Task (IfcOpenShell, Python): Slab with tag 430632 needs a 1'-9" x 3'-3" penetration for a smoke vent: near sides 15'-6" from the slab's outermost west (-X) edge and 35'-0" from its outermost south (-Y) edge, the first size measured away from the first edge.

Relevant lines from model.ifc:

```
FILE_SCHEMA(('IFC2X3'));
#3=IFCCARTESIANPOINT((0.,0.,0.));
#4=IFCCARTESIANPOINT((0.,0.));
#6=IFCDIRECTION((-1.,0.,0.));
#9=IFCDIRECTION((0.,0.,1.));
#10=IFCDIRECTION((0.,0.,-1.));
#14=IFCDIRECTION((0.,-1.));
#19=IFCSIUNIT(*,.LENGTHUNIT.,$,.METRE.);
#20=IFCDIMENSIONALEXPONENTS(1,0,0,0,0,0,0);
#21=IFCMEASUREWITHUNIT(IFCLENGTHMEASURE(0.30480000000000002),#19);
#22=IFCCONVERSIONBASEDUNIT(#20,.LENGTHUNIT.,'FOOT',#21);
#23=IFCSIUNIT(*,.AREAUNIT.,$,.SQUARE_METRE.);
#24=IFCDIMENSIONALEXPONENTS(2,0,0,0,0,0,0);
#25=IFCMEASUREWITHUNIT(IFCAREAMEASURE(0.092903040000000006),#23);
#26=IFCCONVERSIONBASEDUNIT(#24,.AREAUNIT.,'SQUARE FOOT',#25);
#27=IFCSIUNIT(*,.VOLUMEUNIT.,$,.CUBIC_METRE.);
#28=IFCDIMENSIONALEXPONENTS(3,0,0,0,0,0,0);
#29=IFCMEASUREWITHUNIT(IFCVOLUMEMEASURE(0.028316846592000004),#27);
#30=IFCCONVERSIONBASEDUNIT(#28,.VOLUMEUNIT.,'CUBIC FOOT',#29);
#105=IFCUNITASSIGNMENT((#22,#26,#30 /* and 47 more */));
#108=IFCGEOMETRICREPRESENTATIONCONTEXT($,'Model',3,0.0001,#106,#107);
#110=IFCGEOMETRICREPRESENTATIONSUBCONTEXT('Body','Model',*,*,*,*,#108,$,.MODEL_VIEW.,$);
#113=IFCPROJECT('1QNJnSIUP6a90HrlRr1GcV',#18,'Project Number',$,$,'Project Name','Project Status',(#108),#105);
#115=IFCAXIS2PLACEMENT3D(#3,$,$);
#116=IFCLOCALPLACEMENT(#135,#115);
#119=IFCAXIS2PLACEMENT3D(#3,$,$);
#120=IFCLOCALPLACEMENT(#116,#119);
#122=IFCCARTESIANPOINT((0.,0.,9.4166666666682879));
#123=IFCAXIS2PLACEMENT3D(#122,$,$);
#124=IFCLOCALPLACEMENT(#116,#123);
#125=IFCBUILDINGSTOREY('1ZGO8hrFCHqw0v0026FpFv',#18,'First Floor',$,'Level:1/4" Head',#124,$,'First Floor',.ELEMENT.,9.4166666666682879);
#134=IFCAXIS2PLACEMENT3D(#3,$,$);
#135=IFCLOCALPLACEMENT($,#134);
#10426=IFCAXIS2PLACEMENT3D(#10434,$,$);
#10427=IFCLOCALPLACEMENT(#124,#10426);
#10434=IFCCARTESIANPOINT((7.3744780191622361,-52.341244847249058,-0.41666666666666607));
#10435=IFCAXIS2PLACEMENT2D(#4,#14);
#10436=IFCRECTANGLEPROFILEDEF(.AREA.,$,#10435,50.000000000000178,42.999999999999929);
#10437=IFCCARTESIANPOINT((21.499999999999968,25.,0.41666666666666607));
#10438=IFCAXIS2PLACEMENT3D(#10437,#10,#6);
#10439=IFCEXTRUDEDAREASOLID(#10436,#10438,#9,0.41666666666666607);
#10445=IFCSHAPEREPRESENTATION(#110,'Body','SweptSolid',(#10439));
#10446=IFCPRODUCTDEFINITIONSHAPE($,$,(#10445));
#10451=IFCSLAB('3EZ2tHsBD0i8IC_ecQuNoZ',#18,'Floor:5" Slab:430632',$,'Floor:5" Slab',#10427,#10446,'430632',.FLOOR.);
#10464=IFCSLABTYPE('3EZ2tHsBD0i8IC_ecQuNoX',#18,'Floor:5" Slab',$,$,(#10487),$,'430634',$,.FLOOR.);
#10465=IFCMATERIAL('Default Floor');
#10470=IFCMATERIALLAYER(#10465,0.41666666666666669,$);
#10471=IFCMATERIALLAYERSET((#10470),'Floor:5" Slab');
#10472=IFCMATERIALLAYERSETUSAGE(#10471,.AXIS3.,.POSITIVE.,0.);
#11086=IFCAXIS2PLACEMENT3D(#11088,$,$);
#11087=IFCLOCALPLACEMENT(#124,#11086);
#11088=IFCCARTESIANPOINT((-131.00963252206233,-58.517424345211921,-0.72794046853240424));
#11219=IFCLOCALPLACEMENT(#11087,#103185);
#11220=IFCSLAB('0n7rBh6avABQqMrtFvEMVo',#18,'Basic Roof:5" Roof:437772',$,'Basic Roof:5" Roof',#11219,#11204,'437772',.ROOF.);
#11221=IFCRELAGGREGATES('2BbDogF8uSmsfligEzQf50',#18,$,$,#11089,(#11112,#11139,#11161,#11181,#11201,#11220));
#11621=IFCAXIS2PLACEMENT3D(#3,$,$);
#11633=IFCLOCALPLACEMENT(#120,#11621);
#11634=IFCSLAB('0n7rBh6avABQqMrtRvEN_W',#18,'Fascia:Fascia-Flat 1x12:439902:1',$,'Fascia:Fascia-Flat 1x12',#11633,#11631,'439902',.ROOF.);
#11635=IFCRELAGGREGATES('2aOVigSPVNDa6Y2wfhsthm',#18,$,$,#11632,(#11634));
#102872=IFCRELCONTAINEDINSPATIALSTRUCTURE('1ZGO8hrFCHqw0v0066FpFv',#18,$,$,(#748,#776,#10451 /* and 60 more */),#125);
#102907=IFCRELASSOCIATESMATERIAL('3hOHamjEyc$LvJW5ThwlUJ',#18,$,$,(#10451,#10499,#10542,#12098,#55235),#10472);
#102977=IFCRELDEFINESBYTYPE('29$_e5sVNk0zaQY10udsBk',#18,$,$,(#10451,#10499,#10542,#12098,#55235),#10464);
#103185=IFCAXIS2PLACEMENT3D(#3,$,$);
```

```python
import numpy as np
import ifcopenshell
import ifcopenshell.api.feature
import ifcopenshell.api.geometry
import ifcopenshell.api.root
import ifcopenshell.geom
import ifcopenshell.util.placement
import ifcopenshell.util.representation
import ifcopenshell.util.shape
import ifcopenshell.util.unit

model = ifcopenshell.open("model.ifc")
unit_scale = ifcopenshell.util.unit.calculate_unit_scale(model)
settings = ifcopenshell.geom.settings()


def volume(element):
    """Net volume in cubic metres, openings subtracted."""
    shape = ifcopenshell.geom.create_shape(settings, element)
    return ifcopenshell.util.shape.get_volume(shape.geometry)


slab = model.by_guid("3EZ2tHsBD0i8IC_ecQuNoZ")
before = volume(slab)

# Extent in the slab's own axes, in metres. The edges named are its -X and -Y sides.
slab_shape = ifcopenshell.geom.create_shape(settings, slab)
vertices = ifcopenshell.util.shape.get_vertices(slab_shape.geometry)
x_min, y_min, bottom = vertices.min(axis=0)
top = vertices[:, 2].max()

opening = ifcopenshell.api.root.create_entity(model, ifc_class="IfcOpeningElement", name="Smoke vent opening")
context = ifcopenshell.util.representation.get_context(model, "Model", "Body", "MODEL_VIEW")
width, depth = 0.5334, 0.9906
outline = [(0.0, 0.0), (width, 0.0), (width, depth), (0.0, depth), (0.0, 0.0)]
# Overshoot both faces by 50 mm so the cut is clean.
shape = ifcopenshell.api.geometry.add_slab_representation(
    model, context=context, depth=top - bottom + 0.1, polyline=outline
)
ifcopenshell.api.geometry.assign_representation(model, product=opening, representation=shape)

matrix = ifcopenshell.util.placement.get_local_placement(slab.ObjectPlacement)
matrix[:, 3] = matrix @ np.append(np.array([x_min + 4.7244, y_min + 10.668, bottom - 0.05]) / unit_scale, 1.0)
ifcopenshell.api.geometry.edit_object_placement(model, product=opening, matrix=matrix, is_si=False)
ifcopenshell.api.feature.add_feature(model, feature=opening, element=slab)

after = volume(slab)

print(f"slab volume {before:.3f} -> {after:.3f} m3")

model.write("model_updated.ifc")
```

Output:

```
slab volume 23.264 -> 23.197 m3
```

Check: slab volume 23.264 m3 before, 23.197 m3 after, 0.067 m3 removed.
